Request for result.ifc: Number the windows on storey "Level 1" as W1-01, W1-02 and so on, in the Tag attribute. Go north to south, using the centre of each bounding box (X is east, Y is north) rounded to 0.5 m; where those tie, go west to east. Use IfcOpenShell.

First a look at what the model holds.

```python
import ifcopenshell
import ifcopenshell.util.element
import ifcopenshell.util.placement

model = ifcopenshell.open("result.ifc")
print(model.schema)
storey = next(s for s in model.by_type("IfcBuildingStorey") if s.Name == "Level 1")
windows = [e for e in ifcopenshell.util.element.get_decomposition(storey) if e.is_a("IfcWindow")]
for e in sorted(windows, key=lambda e: e.id()):
    origin = ifcopenshell.util.placement.get_local_placement(e.ObjectPlacement)[:3, 3]
    print(e.id(), e.Tag, e.Name, origin.round(2) + 0.0, sep=" | ")
```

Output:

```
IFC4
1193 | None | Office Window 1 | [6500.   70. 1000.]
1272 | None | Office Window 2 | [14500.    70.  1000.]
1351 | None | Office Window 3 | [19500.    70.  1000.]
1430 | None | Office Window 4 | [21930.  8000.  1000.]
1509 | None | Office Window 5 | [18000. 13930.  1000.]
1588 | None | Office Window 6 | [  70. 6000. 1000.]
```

```python
import ifcopenshell
import ifcopenshell.geom
import ifcopenshell.util.element
import ifcopenshell.util.shape

model = ifcopenshell.open("result.ifc")
settings = ifcopenshell.geom.settings()
settings.set("use-world-coords", True)


def centre(element):
    shape = ifcopenshell.geom.create_shape(settings, element)
    return ifcopenshell.util.shape.get_bbox_centroid(shape.geometry)


storey = next(s for s in model.by_type("IfcBuildingStorey") if s.Name == "Level 1")
windows = [e for e in ifcopenshell.util.element.get_decomposition(storey) if e.is_a("IfcWindow")]

# Insertion points can sit at a corner or the storey origin, so sort by the geometry (in metres).
centres = {e: centre(e) for e in windows}
windows.sort(key=lambda e: (-round(centres[e][1] / 0.5), centres[e][0]))

for i, e in enumerate(windows, start=1):
    number = f"W1-{i:02d}"
    e.Tag = number
    print(e.id(), number)

model.write("result-out.ifc")
```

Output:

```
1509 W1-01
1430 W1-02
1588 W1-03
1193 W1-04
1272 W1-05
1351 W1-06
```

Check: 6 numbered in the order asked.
